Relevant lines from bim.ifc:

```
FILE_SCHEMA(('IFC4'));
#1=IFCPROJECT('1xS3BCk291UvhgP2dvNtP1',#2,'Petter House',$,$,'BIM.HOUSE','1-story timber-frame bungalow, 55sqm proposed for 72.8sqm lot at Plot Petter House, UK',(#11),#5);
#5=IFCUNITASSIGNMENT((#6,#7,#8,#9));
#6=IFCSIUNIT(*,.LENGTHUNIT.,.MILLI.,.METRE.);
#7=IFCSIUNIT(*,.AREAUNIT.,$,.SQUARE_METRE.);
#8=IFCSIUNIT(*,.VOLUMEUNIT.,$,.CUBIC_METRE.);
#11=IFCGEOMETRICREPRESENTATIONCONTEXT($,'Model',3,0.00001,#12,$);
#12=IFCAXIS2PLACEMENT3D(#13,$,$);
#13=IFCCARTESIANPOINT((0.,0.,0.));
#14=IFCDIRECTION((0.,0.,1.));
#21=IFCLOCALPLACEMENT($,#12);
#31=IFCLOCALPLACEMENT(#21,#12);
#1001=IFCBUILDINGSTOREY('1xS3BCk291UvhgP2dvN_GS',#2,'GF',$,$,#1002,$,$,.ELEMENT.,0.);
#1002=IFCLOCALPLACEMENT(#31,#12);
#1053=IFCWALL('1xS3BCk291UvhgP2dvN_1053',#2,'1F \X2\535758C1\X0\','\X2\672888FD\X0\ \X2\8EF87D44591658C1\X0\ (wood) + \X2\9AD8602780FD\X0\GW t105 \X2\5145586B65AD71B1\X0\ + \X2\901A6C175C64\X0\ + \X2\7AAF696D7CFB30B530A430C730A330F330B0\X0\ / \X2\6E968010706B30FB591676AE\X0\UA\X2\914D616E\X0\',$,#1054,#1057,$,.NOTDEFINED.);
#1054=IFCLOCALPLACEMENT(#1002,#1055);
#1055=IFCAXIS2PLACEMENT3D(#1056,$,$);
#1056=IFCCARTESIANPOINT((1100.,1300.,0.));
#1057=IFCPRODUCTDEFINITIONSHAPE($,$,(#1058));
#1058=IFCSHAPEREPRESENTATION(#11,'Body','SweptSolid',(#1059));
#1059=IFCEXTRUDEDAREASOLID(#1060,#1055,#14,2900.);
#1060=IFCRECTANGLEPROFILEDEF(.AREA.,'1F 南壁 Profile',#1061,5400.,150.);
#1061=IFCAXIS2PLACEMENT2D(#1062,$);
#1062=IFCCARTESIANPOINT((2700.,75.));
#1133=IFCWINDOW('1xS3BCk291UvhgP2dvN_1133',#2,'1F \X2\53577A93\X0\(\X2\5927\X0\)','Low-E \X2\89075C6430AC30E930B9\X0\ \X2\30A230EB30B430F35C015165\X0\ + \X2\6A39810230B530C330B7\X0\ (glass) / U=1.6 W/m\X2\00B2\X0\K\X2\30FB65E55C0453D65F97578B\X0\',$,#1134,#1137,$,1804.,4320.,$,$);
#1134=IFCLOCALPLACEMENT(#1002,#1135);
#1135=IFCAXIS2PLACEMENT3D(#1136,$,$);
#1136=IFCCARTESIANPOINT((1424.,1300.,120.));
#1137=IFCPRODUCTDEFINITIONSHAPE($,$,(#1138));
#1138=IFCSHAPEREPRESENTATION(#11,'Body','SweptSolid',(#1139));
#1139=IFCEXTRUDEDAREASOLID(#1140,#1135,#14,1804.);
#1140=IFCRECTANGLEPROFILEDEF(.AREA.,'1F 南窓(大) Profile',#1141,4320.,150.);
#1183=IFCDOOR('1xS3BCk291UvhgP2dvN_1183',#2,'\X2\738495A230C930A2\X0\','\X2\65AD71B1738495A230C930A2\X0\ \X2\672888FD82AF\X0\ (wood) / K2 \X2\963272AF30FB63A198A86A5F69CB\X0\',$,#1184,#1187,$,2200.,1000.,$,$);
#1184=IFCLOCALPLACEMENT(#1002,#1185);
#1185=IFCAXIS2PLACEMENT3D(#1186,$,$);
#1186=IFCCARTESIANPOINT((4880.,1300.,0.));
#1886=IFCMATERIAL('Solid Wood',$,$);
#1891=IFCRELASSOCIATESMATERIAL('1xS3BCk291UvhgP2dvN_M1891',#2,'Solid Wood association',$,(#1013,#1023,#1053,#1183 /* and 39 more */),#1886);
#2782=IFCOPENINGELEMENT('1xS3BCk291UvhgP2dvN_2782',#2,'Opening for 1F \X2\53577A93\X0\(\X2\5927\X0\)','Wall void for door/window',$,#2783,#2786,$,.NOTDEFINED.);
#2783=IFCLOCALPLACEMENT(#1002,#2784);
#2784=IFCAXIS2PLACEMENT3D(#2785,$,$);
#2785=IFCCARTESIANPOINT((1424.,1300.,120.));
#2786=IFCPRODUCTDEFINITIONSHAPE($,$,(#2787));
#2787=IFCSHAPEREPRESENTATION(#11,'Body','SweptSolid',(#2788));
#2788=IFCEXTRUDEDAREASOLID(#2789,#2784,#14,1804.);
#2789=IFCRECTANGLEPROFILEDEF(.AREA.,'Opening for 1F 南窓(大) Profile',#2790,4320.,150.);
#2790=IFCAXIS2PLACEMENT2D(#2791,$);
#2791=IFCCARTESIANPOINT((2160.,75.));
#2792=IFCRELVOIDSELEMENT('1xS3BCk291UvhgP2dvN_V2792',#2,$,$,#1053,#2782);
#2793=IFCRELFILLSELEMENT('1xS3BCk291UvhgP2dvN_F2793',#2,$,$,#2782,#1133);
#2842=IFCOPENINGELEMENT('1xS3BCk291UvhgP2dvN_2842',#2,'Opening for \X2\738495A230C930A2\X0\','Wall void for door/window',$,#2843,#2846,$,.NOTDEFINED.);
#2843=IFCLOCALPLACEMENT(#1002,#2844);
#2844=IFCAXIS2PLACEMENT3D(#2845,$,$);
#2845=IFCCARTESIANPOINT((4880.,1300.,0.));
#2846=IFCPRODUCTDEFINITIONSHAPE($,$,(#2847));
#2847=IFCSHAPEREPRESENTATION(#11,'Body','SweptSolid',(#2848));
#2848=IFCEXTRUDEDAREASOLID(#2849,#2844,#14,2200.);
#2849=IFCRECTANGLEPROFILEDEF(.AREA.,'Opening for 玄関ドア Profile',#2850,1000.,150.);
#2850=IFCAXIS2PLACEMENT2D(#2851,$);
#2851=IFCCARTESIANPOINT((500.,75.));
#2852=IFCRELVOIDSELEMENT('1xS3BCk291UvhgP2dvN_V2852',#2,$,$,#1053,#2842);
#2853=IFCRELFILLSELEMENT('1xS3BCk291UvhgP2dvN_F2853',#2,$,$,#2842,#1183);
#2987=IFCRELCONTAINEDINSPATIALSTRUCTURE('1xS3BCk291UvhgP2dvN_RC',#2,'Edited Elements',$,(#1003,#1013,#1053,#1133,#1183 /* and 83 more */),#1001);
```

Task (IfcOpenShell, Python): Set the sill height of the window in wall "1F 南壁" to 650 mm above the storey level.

```python
import numpy as np
import ifcopenshell
import ifcopenshell.api.geometry
import ifcopenshell.geom
import ifcopenshell.util.element
import ifcopenshell.util.placement
import ifcopenshell.util.shape
import ifcopenshell.util.unit

model = ifcopenshell.open("bim.ifc")
unit_scale = ifcopenshell.util.unit.calculate_unit_scale(model)

window = model.by_id(1133)
opening = window.FillsVoids[0].RelatingOpeningElement
storey = ifcopenshell.util.element.get_container(window, ifc_class="IfcBuildingStorey")
level = ifcopenshell.util.placement.get_local_placement(storey.ObjectPlacement)[2, 3]

# The opening's origin need not be at the sill, so measure its lowest point.
shape = ifcopenshell.geom.create_shape(ifcopenshell.geom.settings(), opening)
bottom = ifcopenshell.util.shape.get_shape_bottom_elevation(shape, shape.geometry) / unit_scale
dz = level + 650.0 - bottom

shift = np.array([0.0, 0.0, dz])
# The window is not placed relative to its opening, so move both.
for product in (opening, window):
    matrix = ifcopenshell.util.placement.get_local_placement(product.ObjectPlacement)
    matrix[:3, 3] += shift
    ifcopenshell.api.geometry.edit_object_placement(model, product=product, matrix=matrix, is_si=False)

print(f"moved by {dz * unit_scale:+.3f} m")

model.write("bim_updated.ifc")
```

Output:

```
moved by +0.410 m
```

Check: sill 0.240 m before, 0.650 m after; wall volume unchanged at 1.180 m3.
